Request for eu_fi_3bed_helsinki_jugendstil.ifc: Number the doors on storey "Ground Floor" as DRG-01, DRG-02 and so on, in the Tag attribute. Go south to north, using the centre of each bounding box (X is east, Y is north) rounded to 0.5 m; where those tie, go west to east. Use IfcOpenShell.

First a look at what the model holds.

```python
import ifcopenshell
import ifcopenshell.util.element
import ifcopenshell.util.placement

model = ifcopenshell.open("eu_fi_3bed_helsinki_jugendstil.ifc")
print(model.schema)
storey = next(s for s in model.by_type("IfcBuildingStorey") if s.Name == "Ground Floor")
doors = [e for e in ifcopenshell.util.element.get_decomposition(storey) if e.is_a("IfcDoor")]
for e in sorted(doors, key=lambda e: e.id()):
    origin = ifcopenshell.util.placement.get_local_placement(e.ObjectPlacement)[:3, 3]
    print(e.id(), e.Tag, e.Name, origin.round(2) + 0.0, sep=" | ")
```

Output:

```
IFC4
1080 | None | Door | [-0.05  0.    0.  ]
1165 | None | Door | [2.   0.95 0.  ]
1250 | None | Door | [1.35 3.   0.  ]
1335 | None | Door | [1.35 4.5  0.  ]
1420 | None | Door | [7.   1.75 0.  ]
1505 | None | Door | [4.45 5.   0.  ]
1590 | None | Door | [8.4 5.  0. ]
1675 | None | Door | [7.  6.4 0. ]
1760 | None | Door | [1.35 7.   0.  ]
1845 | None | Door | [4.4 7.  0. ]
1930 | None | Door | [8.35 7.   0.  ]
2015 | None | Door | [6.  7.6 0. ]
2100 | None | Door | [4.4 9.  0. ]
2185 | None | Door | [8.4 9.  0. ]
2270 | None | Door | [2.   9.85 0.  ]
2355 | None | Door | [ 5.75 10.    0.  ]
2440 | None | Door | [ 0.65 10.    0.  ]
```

```python
import ifcopenshell
import ifcopenshell.geom
import ifcopenshell.util.element
import ifcopenshell.util.shape

model = ifcopenshell.open("eu_fi_3bed_helsinki_jugendstil.ifc")
settings = ifcopenshell.geom.settings()
settings.set("use-world-coords", True)


def centre(element):
    shape = ifcopenshell.geom.create_shape(settings, element)
    return ifcopenshell.util.shape.get_bbox_centroid(shape.geometry)


storey = next(s for s in model.by_type("IfcBuildingStorey") if s.Name == "Ground Floor")
doors = [e for e in ifcopenshell.util.element.get_decomposition(storey) if e.is_a("IfcDoor")]

# Insertion points can sit at a corner or the storey origin, so sort by the geometry (in metres).
centres = {e: centre(e) for e in doors}
doors.sort(key=lambda e: (round(centres[e][1] / 0.5), centres[e][0]))

for i, e in enumerate(doors, start=1):
    number = f"DRG-{i:02d}"
    e.Tag = number
    print(e.id(), number)

model.write("eu_fi_3bed_helsinki_jugendstil_rev.ifc")
```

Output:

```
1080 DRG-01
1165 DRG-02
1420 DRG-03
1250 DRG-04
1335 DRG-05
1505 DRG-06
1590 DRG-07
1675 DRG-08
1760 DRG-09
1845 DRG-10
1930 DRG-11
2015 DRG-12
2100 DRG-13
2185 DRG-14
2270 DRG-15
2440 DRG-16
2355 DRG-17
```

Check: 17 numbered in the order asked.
